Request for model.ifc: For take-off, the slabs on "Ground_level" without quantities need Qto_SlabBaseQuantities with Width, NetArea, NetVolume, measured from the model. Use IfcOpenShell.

First a look at what the model holds.

```python
import ifcopenshell
import ifcopenshell.util.element
import ifcopenshell.util.unit

model = ifcopenshell.open("model.ifc")
print(model.schema)
for unit_type in ("LENGTHUNIT", "AREAUNIT", "VOLUMEUNIT"):
    print(unit_type, ifcopenshell.util.unit.calculate_unit_scale(model, unit_type))
storey = next(s for s in model.by_type("IfcBuildingStorey") if s.Name == "Ground_level")
slabs = [e for e in ifcopenshell.util.element.get_decomposition(storey) if e.is_a("IfcSlab")]
for e in sorted(slabs, key=lambda e: e.id()):
    print(e.id(), e.is_a(), e.Name, list(ifcopenshell.util.element.get_psets(e, qtos_only=True)), sep=" | ")
```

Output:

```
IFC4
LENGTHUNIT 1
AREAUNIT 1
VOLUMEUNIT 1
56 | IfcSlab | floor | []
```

```python
import ifcopenshell
import ifcopenshell.api.pset
import ifcopenshell.geom
import ifcopenshell.util.element
import ifcopenshell.util.shape
import ifcopenshell.util.unit

model = ifcopenshell.open("model.ifc")
unit_scale = ifcopenshell.util.unit.calculate_unit_scale(model)
area_scale = ifcopenshell.util.unit.calculate_unit_scale(model, "AREAUNIT")
volume_scale = ifcopenshell.util.unit.calculate_unit_scale(model, "VOLUMEUNIT")
settings = ifcopenshell.geom.settings()

storey = next(s for s in model.by_type("IfcBuildingStorey") if s.Name == "Ground_level")
slabs = [e for e in ifcopenshell.util.element.get_decomposition(storey) if e.is_a("IfcSlab")]

for e in sorted(slabs, key=lambda e: e.id()):
    if ifcopenshell.util.element.get_psets(e, qtos_only=True, should_inherit=False):
        continue
    # Geometry comes back in metres, in the element's own axes.
    shape = ifcopenshell.geom.create_shape(settings, e)
    values = {
        "Width": ifcopenshell.util.shape.get_z(shape.geometry) / unit_scale,
        "NetArea": ifcopenshell.util.shape.get_footprint_area(shape.geometry) / area_scale,
        "NetVolume": ifcopenshell.util.shape.get_volume(shape.geometry) / volume_scale,
    }
    qto = ifcopenshell.api.pset.add_qto(model, product=e, name="Qto_SlabBaseQuantities")
    ifcopenshell.api.pset.edit_qto(model, qto=qto, properties=values)
    print(e.id(), {k: round(v, 3) for k, v in values.items()})

model.write("model_v2.ifc")
```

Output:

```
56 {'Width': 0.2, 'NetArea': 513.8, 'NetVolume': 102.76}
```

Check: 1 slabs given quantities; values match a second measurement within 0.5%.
